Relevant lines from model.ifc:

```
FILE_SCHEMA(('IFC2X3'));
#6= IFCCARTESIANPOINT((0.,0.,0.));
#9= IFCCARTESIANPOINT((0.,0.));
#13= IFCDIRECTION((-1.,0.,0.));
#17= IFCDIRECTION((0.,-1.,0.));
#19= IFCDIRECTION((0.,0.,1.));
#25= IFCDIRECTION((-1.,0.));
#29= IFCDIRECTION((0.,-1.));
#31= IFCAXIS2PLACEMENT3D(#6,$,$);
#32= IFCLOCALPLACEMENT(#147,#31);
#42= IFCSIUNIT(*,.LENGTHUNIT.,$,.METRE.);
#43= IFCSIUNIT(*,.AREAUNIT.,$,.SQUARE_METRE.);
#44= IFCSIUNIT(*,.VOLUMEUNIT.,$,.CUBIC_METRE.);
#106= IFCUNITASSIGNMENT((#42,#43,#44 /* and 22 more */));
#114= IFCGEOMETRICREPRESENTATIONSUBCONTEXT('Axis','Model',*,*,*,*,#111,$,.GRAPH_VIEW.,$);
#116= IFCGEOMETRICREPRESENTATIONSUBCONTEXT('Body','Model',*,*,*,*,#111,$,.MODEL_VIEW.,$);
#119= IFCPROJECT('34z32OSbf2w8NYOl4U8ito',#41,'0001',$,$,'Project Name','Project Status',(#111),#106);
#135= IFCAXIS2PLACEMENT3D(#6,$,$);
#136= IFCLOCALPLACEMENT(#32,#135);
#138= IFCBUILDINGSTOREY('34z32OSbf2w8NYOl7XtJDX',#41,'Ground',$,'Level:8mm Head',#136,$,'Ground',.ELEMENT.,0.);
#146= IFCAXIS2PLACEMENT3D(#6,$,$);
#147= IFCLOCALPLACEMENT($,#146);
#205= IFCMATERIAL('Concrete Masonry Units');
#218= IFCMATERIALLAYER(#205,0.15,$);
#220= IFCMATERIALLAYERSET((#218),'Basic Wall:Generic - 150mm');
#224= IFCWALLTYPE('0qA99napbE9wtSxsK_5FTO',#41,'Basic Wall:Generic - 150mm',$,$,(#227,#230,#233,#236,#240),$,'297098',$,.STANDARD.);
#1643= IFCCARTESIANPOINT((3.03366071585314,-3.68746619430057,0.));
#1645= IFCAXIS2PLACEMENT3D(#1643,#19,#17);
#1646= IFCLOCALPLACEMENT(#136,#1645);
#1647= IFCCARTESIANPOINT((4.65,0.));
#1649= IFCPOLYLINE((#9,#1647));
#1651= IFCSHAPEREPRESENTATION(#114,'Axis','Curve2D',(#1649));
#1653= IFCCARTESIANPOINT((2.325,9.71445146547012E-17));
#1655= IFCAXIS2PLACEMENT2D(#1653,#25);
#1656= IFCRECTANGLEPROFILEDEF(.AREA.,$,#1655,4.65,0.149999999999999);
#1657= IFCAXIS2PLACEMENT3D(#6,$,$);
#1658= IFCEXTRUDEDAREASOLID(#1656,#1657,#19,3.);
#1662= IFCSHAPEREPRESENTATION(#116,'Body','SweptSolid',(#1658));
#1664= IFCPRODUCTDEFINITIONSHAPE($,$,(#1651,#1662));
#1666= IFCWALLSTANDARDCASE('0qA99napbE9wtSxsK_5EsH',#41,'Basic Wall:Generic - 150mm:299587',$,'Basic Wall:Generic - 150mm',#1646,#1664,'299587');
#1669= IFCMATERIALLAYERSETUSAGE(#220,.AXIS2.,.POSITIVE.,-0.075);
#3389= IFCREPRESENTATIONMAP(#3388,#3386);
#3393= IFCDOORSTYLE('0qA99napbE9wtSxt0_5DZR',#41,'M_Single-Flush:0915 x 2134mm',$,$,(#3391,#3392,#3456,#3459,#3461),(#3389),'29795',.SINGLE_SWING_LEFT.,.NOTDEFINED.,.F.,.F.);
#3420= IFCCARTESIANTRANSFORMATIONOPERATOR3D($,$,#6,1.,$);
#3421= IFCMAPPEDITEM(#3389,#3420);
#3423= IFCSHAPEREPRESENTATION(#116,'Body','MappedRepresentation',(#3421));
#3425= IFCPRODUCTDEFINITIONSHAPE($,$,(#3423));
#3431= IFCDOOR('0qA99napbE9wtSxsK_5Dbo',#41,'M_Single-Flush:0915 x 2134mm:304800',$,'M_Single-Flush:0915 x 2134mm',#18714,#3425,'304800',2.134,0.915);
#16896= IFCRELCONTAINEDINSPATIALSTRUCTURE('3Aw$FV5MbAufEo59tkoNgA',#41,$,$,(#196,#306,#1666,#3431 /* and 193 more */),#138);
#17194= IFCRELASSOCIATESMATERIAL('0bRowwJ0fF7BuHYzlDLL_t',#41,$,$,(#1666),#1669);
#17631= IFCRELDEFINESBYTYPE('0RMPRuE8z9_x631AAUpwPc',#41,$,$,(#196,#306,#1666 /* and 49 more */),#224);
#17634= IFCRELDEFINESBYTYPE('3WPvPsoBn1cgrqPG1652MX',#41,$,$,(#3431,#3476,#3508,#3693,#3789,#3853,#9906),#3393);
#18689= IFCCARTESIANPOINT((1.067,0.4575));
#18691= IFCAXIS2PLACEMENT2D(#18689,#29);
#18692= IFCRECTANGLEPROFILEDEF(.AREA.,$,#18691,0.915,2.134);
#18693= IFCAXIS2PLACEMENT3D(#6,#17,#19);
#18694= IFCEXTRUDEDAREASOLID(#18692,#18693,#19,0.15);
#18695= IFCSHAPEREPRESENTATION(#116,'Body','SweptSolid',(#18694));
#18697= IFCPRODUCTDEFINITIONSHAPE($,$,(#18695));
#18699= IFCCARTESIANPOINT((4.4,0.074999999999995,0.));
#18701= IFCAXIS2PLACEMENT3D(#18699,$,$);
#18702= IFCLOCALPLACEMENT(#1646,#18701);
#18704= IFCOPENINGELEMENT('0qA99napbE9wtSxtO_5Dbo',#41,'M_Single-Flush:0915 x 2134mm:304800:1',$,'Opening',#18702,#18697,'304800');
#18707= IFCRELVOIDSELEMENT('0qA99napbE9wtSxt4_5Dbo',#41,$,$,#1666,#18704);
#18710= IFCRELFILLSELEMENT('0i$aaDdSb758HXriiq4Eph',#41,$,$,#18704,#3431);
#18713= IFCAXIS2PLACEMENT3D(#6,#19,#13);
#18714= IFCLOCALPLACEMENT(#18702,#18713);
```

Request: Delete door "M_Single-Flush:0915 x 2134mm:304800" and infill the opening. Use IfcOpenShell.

```python
import ifcopenshell
import ifcopenshell.api.feature
import ifcopenshell.api.root
import ifcopenshell.geom
import ifcopenshell.util.shape

model = ifcopenshell.open("model.ifc")
settings = ifcopenshell.geom.settings()


def volume(element):
    """Net volume in cubic metres, openings subtracted."""
    shape = ifcopenshell.geom.create_shape(settings, element)
    return ifcopenshell.util.shape.get_volume(shape.geometry)


door = model.by_guid("0qA99napbE9wtSxsK_5Dbo")
opening = door.FillsVoids[0].RelatingOpeningElement
wall = opening.VoidsElements[0].RelatingBuildingElement
before = volume(wall)

ifcopenshell.api.root.remove_product(model, product=door)
ifcopenshell.api.feature.remove_feature(model, feature=opening)

after = volume(wall)

print(f"wall volume {before:.3f} -> {after:.3f} m3")

model.write("model_rev.ifc")
```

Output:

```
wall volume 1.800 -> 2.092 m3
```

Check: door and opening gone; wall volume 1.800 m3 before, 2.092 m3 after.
